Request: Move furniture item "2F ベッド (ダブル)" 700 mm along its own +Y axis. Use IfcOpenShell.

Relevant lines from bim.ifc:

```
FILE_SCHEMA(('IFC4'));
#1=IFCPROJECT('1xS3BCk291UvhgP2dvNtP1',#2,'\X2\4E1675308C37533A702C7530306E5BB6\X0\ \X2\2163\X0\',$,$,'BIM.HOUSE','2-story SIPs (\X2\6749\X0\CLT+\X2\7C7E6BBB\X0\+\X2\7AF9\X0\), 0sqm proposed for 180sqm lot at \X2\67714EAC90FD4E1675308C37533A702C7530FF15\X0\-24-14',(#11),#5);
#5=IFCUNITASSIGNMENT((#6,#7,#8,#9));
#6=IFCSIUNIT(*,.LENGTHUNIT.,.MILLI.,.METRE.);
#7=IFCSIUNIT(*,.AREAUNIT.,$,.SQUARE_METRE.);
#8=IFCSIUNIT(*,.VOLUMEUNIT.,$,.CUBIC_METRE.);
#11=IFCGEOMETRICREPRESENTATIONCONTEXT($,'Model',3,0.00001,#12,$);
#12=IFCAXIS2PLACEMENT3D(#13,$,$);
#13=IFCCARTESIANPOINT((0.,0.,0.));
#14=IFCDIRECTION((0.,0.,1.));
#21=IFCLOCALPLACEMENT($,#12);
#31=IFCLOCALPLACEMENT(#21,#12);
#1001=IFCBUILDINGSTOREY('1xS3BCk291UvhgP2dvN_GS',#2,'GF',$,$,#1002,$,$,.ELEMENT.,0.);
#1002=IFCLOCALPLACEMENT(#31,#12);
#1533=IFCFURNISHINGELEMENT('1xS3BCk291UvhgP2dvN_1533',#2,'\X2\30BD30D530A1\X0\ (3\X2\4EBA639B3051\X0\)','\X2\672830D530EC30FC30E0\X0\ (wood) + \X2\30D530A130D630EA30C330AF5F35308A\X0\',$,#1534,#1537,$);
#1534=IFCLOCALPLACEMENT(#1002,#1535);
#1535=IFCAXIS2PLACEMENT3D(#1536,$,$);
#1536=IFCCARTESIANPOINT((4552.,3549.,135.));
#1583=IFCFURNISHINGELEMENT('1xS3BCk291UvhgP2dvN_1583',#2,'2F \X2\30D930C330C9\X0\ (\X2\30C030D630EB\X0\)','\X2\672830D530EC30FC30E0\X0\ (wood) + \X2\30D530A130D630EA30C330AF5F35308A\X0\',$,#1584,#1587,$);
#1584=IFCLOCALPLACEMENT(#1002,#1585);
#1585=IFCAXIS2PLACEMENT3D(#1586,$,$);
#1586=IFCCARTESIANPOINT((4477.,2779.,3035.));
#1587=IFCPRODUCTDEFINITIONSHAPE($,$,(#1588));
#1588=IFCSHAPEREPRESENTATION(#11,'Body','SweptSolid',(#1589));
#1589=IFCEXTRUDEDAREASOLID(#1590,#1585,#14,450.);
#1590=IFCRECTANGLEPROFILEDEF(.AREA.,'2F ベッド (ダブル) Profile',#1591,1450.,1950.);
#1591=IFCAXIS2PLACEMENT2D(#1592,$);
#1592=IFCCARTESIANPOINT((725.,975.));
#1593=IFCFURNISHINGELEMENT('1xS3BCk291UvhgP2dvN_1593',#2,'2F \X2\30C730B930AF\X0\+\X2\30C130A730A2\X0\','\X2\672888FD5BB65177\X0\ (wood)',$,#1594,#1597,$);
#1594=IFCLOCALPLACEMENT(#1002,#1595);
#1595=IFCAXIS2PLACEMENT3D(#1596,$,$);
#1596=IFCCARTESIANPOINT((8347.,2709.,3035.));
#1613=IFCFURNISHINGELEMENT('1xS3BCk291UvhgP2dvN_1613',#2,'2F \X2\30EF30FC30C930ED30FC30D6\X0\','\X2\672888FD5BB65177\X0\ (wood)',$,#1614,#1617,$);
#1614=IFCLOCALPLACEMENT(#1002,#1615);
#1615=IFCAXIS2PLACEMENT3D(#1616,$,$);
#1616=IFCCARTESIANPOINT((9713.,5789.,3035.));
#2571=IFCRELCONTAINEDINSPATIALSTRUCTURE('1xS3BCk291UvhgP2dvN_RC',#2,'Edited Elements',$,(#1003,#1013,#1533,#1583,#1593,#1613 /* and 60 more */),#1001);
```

```python
import ifcopenshell
import ifcopenshell.api.geometry
import ifcopenshell.util.placement

model = ifcopenshell.open("bim.ifc")

item = model.by_id(1583)
matrix = ifcopenshell.util.placement.get_local_placement(item.ObjectPlacement)
matrix[:3, 3] += matrix[:3, 1] * 700.0
ifcopenshell.api.geometry.edit_object_placement(model, product=item, matrix=matrix, is_si=False)

print(ifcopenshell.util.placement.get_local_placement(item.ObjectPlacement).round(3) + 0.0)

model.write("bim_rev.ifc")
```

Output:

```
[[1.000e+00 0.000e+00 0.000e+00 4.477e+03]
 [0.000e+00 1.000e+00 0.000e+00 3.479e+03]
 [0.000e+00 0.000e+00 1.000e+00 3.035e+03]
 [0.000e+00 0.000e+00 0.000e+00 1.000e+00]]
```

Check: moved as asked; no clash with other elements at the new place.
